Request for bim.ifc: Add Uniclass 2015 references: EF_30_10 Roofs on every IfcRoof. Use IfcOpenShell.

First a look at what the model holds.

```python
import ifcopenshell

model = ifcopenshell.open("bim.ifc")
print(model.schema)
print("classifications:", [c.Name for c in model.by_type("IfcClassification")])
for ifc_class in ("IfcDoor", "IfcRoof", "IfcStair", "IfcWall", "IfcWindow"):
    print(ifc_class, len(model.by_type(ifc_class)))
```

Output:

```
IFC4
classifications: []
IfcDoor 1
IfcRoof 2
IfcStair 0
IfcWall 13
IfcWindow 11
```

```python
import ifcopenshell
import ifcopenshell.api.classification

model = ifcopenshell.open("bim.ifc")

system = ifcopenshell.api.classification.add_classification(model, classification="Uniclass 2015")

codes = {
    "IfcRoof": ("EF_30_10", "Roofs"),
}
for ifc_class, (code, name) in codes.items():
    products = model.by_type(ifc_class)
    ifcopenshell.api.classification.add_reference(
        model, products=products, classification=system, identification=code, name=name
    )
    print(code, len(products))

model.write("bim_v2.ifc")
```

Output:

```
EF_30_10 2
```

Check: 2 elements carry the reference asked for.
